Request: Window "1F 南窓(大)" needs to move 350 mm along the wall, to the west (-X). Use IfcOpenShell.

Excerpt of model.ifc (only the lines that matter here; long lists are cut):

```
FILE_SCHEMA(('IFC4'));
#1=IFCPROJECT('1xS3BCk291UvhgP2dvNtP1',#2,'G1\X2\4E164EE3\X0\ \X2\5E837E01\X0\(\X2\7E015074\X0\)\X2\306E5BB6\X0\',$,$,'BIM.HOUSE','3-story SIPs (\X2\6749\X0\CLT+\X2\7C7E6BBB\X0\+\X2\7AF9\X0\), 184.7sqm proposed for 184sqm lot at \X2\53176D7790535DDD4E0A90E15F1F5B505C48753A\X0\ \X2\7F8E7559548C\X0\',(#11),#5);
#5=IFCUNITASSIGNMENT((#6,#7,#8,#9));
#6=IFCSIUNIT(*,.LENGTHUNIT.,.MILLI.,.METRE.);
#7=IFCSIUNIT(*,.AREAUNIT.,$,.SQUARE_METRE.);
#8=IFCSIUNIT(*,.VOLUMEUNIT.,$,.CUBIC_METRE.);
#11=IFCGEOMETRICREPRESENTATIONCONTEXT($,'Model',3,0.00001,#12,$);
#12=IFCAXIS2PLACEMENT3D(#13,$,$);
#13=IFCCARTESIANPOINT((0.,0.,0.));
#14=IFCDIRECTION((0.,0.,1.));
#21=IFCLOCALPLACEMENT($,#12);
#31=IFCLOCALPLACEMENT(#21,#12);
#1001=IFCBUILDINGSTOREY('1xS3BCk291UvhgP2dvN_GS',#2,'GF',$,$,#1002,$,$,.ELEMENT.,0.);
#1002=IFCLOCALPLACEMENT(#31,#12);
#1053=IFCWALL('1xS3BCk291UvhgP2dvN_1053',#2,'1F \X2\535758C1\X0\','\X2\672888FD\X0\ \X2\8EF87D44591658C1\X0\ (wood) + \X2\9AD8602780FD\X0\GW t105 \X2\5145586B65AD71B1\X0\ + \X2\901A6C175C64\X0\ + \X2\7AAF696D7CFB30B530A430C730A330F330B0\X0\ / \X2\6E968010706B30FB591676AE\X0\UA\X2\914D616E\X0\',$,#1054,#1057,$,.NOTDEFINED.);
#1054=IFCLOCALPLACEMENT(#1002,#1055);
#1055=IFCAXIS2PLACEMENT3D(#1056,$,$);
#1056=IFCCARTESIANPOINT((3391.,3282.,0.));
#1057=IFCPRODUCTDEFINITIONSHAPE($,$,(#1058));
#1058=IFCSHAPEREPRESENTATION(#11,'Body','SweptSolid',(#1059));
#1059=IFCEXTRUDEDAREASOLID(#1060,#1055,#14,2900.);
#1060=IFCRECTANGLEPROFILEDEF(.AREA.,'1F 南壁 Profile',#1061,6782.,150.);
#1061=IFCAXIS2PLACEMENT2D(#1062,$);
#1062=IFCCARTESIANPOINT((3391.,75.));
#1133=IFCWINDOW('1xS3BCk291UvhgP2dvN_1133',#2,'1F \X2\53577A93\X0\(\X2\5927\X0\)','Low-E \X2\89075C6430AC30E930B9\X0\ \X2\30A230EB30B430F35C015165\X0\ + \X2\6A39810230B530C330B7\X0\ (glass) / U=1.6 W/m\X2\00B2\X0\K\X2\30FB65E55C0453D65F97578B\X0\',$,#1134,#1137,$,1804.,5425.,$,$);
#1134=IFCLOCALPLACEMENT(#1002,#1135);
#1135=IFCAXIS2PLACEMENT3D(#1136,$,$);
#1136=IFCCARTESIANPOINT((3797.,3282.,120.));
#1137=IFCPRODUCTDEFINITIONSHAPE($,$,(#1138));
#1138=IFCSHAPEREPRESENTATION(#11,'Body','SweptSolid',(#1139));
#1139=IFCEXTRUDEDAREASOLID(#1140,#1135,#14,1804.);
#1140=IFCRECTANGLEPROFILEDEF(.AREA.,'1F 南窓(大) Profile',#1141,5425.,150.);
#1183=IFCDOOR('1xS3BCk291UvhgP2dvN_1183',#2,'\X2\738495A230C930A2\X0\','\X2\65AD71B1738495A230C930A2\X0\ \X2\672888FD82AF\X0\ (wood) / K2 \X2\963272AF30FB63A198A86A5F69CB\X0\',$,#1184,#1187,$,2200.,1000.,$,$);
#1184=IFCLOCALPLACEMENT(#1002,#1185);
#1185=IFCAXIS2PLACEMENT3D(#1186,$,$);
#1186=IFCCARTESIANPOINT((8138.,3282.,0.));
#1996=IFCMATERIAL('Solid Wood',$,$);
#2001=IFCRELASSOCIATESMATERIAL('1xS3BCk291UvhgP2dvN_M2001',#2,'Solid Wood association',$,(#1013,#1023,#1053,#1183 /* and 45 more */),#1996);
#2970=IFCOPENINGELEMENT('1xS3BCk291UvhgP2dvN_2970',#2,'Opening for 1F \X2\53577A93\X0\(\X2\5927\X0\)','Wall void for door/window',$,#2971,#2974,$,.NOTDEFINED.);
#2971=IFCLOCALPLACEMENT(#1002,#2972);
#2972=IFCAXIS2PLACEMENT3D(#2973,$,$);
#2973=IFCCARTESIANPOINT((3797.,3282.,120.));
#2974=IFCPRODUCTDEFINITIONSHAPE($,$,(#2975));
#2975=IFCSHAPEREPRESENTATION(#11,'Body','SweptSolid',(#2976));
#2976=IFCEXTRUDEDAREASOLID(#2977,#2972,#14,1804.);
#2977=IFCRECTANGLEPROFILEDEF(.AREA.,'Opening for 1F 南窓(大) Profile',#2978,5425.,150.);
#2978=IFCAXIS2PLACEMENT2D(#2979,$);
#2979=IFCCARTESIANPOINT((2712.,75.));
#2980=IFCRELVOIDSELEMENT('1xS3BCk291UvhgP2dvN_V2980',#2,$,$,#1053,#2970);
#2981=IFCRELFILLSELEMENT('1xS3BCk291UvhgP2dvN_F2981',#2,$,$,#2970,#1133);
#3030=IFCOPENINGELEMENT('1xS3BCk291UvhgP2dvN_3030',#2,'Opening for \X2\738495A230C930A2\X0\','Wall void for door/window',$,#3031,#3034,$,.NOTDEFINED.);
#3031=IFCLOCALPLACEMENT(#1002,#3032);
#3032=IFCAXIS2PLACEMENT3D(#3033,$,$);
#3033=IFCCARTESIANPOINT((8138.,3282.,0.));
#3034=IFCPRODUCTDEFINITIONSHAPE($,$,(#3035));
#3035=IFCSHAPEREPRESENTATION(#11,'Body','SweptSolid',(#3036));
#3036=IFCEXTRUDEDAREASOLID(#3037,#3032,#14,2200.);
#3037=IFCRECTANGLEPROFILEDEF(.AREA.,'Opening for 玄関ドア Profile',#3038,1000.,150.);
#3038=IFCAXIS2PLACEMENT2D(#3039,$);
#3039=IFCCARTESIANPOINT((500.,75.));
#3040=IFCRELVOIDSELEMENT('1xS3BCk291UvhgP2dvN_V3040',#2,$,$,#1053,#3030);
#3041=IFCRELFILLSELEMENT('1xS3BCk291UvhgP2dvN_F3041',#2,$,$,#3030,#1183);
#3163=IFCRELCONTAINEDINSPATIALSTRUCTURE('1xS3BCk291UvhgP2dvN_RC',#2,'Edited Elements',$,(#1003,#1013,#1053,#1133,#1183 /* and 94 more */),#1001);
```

```python
import ifcopenshell
import ifcopenshell.api.geometry
import ifcopenshell.util.placement

model = ifcopenshell.open("model.ifc")

window = model.by_guid("1xS3BCk291UvhgP2dvN_1133")
opening = window.FillsVoids[0].RelatingOpeningElement
wall = opening.VoidsElements[0].RelatingBuildingElement

wall_matrix = ifcopenshell.util.placement.get_local_placement(wall.ObjectPlacement)
shift = wall_matrix[:3, 0] * -350.0
before = ifcopenshell.util.placement.get_local_placement(window.ObjectPlacement)[:3, 3].copy()

# The window is not placed relative to its opening, so move both.
for product in (opening, window):
    matrix = ifcopenshell.util.placement.get_local_placement(product.ObjectPlacement)
    matrix[:3, 3] += shift
    ifcopenshell.api.geometry.edit_object_placement(model, product=product, matrix=matrix, is_si=False)

after = ifcopenshell.util.placement.get_local_placement(window.ObjectPlacement)[:3, 3]
print("window moved by", (after - before).round(3) + 0.0)

model.write("model_v2.ifc")
```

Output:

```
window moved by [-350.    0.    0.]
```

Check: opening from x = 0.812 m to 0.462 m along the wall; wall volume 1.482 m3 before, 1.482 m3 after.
